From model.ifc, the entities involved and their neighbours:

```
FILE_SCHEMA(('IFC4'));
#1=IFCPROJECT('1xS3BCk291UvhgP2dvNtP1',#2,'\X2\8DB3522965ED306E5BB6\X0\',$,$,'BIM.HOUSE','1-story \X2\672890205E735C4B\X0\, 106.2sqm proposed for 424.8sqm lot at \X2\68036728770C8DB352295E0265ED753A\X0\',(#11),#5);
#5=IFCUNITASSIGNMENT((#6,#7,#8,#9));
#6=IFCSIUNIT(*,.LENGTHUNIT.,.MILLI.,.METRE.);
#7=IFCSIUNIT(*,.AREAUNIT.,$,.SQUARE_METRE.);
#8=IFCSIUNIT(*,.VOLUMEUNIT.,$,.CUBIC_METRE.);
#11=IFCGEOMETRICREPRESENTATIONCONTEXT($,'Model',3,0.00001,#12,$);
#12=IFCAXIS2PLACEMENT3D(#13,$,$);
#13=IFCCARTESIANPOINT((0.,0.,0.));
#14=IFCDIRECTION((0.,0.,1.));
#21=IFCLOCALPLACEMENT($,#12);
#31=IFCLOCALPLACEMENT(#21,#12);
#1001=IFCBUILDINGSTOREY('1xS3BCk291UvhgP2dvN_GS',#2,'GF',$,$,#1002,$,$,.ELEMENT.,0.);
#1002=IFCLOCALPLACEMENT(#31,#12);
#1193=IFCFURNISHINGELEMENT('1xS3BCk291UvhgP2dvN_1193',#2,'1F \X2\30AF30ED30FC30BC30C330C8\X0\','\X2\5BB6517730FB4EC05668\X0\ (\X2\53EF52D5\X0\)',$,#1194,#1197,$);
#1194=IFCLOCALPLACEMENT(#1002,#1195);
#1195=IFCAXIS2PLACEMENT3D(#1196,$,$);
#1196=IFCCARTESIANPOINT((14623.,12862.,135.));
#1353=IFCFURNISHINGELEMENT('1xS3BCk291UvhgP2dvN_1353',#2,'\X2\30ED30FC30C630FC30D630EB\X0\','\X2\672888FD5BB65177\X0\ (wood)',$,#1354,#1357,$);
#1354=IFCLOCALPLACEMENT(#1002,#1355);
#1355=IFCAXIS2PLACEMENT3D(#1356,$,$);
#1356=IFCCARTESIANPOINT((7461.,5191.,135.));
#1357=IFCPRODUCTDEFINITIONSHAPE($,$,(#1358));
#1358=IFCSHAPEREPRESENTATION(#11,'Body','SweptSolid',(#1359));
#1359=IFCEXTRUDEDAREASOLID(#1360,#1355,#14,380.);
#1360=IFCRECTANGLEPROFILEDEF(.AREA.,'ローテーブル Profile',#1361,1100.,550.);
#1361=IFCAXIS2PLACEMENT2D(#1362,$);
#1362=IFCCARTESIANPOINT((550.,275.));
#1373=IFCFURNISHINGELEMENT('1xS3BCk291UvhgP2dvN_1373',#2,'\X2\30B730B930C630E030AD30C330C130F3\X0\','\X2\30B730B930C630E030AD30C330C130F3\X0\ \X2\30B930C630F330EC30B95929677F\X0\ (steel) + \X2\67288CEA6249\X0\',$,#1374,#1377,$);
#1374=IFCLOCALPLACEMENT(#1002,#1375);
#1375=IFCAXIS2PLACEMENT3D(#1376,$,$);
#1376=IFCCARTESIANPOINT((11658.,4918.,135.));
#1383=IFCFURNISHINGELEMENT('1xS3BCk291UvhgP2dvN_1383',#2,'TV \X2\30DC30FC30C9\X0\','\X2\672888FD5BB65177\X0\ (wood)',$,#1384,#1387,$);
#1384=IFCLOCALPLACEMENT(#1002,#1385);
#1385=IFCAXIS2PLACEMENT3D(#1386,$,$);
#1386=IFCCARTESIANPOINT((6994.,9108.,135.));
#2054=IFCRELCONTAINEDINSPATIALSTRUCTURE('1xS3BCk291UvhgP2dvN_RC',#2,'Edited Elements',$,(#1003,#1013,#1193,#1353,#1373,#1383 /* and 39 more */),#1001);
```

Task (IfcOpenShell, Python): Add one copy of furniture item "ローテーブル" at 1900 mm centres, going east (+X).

```python
import numpy as np
import ifcopenshell
import ifcopenshell.api.geometry
import ifcopenshell.api.root
import ifcopenshell.util.element
import ifcopenshell.util.placement

model = ifcopenshell.open("model.ifc")


def reuse_history(source, copy):
    """copy_class also copies each property set's owner history, people and application; keep the originals."""
    for rel in copy.IsDefinedBy:
        if rel.is_a("IfcRelDefinesByProperties") and (history := rel.RelatingPropertyDefinition.OwnerHistory):
            rel.RelatingPropertyDefinition.OwnerHistory = source.OwnerHistory
            ifcopenshell.util.element.remove_deep2(model, history)


source = model.by_id(1353)
base = ifcopenshell.util.placement.get_local_placement(source.ObjectPlacement)
step = np.array([1.0, 0.0, 0.0]) * 1900.0

for i in range(1, 2):
    copy = ifcopenshell.api.root.copy_class(model, product=source)
    copy.Representation = ifcopenshell.util.element.copy_deep(
        model, source.Representation, exclude=["IfcGeometricRepresentationContext", "IfcRepresentationMap"]
    )
    reuse_history(source, copy)
    matrix = base.copy()
    matrix[:3, 3] += i * step
    print("added at", matrix[:3, 3].round(3) + 0.0)
    ifcopenshell.api.geometry.edit_object_placement(model, product=copy, matrix=matrix, is_si=False)

model.write("model_updated.ifc")
```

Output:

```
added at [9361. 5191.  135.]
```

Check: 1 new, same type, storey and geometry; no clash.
